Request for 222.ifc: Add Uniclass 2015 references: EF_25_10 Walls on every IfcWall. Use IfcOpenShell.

First a look at what the model holds.

```python
import ifcopenshell

model = ifcopenshell.open("222.ifc")
print(model.schema)
print("classifications:", [c.Name for c in model.by_type("IfcClassification")])
for ifc_class in ("IfcDoor", "IfcRoof", "IfcStair", "IfcWall", "IfcWindow"):
    print(ifc_class, len(model.by_type(ifc_class)))
```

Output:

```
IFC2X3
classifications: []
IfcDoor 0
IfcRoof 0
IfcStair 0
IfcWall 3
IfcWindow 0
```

```python
import ifcopenshell
import ifcopenshell.api.classification

model = ifcopenshell.open("222.ifc")

# IFC2X3 requires Source and Edition and has no link from the project to the system.
system = model.create_entity("IfcClassification", Source="NBS", Edition="2015", Name="Uniclass 2015")

codes = {
    "IfcWall": ("EF_25_10", "Walls"),
}
for ifc_class, (code, name) in codes.items():
    products = model.by_type(ifc_class)
    ifcopenshell.api.classification.add_reference(
        model, products=products, classification=system, identification=code, name=name
    )
    print(code, len(products))

model.write("222_v2.ifc")
```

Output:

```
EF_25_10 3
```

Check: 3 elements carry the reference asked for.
